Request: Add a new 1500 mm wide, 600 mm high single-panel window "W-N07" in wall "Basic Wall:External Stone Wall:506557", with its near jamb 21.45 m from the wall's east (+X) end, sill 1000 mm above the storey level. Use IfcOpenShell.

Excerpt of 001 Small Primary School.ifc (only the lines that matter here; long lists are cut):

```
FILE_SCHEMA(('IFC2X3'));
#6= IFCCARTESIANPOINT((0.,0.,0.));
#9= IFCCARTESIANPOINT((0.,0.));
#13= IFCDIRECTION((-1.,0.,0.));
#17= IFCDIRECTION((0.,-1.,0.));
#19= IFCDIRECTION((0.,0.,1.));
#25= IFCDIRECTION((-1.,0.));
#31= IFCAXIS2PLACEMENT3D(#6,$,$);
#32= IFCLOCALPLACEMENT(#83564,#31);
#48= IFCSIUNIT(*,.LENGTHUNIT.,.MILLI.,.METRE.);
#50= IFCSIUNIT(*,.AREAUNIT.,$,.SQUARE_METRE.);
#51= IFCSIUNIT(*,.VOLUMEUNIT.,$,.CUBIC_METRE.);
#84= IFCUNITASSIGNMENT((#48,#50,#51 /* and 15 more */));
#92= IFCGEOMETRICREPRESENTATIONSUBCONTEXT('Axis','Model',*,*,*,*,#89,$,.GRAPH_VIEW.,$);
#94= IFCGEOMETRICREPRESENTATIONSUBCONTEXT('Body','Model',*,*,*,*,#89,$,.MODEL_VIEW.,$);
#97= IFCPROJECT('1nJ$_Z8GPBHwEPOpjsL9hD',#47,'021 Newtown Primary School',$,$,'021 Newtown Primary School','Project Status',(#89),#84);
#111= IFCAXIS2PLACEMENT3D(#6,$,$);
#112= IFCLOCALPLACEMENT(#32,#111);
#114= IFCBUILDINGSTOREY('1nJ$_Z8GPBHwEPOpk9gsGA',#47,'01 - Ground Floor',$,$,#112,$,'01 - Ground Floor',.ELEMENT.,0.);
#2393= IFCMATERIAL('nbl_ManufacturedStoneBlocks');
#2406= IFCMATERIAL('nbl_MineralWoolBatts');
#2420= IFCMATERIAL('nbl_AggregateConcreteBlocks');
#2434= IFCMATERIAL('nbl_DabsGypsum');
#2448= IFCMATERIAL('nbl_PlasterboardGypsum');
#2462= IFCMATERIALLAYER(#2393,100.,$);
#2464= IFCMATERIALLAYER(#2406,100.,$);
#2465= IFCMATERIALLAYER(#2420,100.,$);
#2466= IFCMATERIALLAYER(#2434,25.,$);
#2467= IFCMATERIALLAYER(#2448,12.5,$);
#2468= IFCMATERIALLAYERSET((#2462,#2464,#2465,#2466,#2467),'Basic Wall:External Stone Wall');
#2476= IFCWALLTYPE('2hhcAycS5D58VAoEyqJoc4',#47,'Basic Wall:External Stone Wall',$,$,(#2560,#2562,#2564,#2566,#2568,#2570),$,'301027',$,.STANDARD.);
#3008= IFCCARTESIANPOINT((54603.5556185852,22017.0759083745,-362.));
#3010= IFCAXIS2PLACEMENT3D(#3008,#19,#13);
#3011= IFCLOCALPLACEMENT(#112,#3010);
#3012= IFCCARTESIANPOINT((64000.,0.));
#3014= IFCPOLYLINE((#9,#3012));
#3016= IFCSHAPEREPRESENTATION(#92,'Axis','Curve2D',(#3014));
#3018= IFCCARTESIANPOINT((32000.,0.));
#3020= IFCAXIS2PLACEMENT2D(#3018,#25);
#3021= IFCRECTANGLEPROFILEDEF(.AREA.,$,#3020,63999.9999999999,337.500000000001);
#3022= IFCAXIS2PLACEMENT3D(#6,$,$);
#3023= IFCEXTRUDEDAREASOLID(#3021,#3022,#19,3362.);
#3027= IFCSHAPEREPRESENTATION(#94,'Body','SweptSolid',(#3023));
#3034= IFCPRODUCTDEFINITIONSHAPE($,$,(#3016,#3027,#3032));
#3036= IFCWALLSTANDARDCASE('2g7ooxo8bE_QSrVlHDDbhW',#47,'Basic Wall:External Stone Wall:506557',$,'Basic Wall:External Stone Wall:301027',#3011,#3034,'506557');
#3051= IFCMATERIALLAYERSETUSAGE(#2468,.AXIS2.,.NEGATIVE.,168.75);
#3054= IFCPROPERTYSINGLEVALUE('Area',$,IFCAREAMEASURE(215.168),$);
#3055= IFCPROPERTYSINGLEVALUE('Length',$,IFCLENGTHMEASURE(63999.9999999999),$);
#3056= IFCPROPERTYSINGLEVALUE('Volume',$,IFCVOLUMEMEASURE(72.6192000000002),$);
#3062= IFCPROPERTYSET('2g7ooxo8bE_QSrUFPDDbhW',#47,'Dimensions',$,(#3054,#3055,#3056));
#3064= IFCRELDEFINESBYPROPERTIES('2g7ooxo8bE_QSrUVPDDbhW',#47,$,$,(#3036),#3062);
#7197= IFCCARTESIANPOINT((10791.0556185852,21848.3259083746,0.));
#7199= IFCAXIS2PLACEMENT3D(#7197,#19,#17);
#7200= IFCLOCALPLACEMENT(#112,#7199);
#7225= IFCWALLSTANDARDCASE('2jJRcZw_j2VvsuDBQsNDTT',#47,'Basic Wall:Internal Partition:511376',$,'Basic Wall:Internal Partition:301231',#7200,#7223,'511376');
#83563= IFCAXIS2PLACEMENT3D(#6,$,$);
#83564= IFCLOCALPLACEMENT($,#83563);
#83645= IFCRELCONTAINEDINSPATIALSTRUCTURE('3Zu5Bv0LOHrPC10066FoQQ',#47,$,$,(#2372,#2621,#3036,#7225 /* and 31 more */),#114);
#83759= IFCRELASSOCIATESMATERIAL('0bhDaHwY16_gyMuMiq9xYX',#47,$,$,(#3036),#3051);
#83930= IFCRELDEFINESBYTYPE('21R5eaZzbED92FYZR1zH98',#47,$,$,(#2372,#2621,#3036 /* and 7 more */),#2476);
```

```python
import numpy as np
import ifcopenshell
import ifcopenshell.api.feature
import ifcopenshell.api.geometry
import ifcopenshell.api.pset
import ifcopenshell.api.root
import ifcopenshell.api.spatial
import ifcopenshell.api.type
import ifcopenshell.geom
import ifcopenshell.util.element
import ifcopenshell.util.placement
import ifcopenshell.util.representation
import ifcopenshell.util.shape
import ifcopenshell.util.unit

model = ifcopenshell.open("001 Small Primary School.ifc")
unit_scale = ifcopenshell.util.unit.calculate_unit_scale(model)
area_scale = ifcopenshell.util.unit.calculate_unit_scale(model, "AREAUNIT")
volume_scale = ifcopenshell.util.unit.calculate_unit_scale(model, "VOLUMEUNIT")
settings = ifcopenshell.geom.settings()


def volume(element):
    """Net volume in cubic metres, openings subtracted."""
    shape = ifcopenshell.geom.create_shape(settings, element)
    return ifcopenshell.util.shape.get_volume(shape.geometry)


wall = model.by_guid("2g7ooxo8bE_QSrVlHDDbhW")
storey = ifcopenshell.util.element.get_container(wall, ifc_class="IfcBuildingStorey")
context = ifcopenshell.util.representation.get_context(model, "Model", "Body", "MODEL_VIEW")
before = volume(wall)

width, height, from_end, sill = 1.5, 0.6, 21.45, 1  # metres

# The wall runs along its own X axis, and the end named is its -X end.
wall_shape = ifcopenshell.geom.create_shape(settings, wall)
x, y, z = ifcopenshell.util.shape.get_vertices(wall_shape.geometry).T
start = x.min() + from_end
face, thickness = float(y.min()), float(y.max() - y.min())
wall_matrix = ifcopenshell.util.placement.get_local_placement(wall.ObjectPlacement)
level = ifcopenshell.util.placement.get_local_placement(storey.ObjectPlacement)[2, 3]


def in_wall(x, y):
    """Placement at x, y metres in the wall's axes, at sill height."""
    matrix = wall_matrix.copy()
    matrix[:, 3] = wall_matrix @ np.array([x / unit_scale, y / unit_scale, 0.0, 1.0])
    matrix[2, 3] = level + sill / unit_scale
    return matrix


# Opening: a box that overshoots both wall faces by 50 mm.
opening = ifcopenshell.api.root.create_entity(model, ifc_class="IfcOpeningElement")
box = ifcopenshell.api.geometry.add_wall_representation(
    model, context=context, length=width, height=height, thickness=thickness + 0.1
)
ifcopenshell.api.geometry.assign_representation(model, product=opening, representation=box)
ifcopenshell.api.geometry.edit_object_placement(model, product=opening, matrix=in_wall(start, face - 0.05), is_si=False)
ifcopenshell.api.feature.add_feature(model, feature=opening, element=wall)

window = ifcopenshell.api.root.create_entity(model, ifc_class="IfcWindow", name="W-N07")
window.OverallWidth, window.OverallHeight = width / unit_scale, height / unit_scale
body = ifcopenshell.api.geometry.add_window_representation(
    model,
    context=context,
    overall_width=window.OverallWidth,
    overall_height=window.OverallHeight,
    partition_type="SINGLE_PANEL",
)
ifcopenshell.api.geometry.assign_representation(model, product=window, representation=body)
ifcopenshell.api.spatial.assign_container(model, products=[window], relating_structure=storey)
fills = ifcopenshell.api.feature.add_filling(model, opening=opening, element=window)
fills.OwnerHistory = window.OwnerHistory  # required in IFC2X3

# IFC2X3 keeps the operation on the window style.
style = ifcopenshell.api.root.create_entity(model, ifc_class="IfcWindowStyle", name="W-N07")
style.OperationType, style.ConstructionType = "SINGLE_PANEL", "NOTDEFINED"
style.ParameterTakesPrecedence = style.Sizeable = False
ifcopenshell.api.type.assign_type(model, related_objects=[window], relating_type=style)

# Centre the window in the wall's thickness.
ifcopenshell.api.geometry.edit_object_placement(model, product=window, matrix=in_wall(start, face), is_si=False)
window_shape = ifcopenshell.geom.create_shape(settings, window)
depth = ifcopenshell.util.shape.get_vertices(window_shape.geometry)[:, 1]
offset = face + thickness / 2 - (depth.min() + depth.max()) / 2
ifcopenshell.api.geometry.edit_object_placement(model, product=window, matrix=in_wall(start, offset), is_si=False)

after = volume(wall)

# Update the wall's stored quantities.
pset = model.by_id(ifcopenshell.util.element.get_pset(wall, "Dimensions", should_inherit=False)["id"])
ifcopenshell.api.pset.edit_pset(model, pset=pset, properties={
    "Area": model.create_entity("IfcAreaMeasure", after / thickness / area_scale),
    "Volume": model.create_entity("IfcVolumeMeasure", after / volume_scale),
})

print(f"wall volume {before:.3f} -> {after:.3f} m3")

model.write("001 Small Primary School_edited.ifc")
```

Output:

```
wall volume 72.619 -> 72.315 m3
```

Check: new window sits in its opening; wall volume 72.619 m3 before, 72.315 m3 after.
